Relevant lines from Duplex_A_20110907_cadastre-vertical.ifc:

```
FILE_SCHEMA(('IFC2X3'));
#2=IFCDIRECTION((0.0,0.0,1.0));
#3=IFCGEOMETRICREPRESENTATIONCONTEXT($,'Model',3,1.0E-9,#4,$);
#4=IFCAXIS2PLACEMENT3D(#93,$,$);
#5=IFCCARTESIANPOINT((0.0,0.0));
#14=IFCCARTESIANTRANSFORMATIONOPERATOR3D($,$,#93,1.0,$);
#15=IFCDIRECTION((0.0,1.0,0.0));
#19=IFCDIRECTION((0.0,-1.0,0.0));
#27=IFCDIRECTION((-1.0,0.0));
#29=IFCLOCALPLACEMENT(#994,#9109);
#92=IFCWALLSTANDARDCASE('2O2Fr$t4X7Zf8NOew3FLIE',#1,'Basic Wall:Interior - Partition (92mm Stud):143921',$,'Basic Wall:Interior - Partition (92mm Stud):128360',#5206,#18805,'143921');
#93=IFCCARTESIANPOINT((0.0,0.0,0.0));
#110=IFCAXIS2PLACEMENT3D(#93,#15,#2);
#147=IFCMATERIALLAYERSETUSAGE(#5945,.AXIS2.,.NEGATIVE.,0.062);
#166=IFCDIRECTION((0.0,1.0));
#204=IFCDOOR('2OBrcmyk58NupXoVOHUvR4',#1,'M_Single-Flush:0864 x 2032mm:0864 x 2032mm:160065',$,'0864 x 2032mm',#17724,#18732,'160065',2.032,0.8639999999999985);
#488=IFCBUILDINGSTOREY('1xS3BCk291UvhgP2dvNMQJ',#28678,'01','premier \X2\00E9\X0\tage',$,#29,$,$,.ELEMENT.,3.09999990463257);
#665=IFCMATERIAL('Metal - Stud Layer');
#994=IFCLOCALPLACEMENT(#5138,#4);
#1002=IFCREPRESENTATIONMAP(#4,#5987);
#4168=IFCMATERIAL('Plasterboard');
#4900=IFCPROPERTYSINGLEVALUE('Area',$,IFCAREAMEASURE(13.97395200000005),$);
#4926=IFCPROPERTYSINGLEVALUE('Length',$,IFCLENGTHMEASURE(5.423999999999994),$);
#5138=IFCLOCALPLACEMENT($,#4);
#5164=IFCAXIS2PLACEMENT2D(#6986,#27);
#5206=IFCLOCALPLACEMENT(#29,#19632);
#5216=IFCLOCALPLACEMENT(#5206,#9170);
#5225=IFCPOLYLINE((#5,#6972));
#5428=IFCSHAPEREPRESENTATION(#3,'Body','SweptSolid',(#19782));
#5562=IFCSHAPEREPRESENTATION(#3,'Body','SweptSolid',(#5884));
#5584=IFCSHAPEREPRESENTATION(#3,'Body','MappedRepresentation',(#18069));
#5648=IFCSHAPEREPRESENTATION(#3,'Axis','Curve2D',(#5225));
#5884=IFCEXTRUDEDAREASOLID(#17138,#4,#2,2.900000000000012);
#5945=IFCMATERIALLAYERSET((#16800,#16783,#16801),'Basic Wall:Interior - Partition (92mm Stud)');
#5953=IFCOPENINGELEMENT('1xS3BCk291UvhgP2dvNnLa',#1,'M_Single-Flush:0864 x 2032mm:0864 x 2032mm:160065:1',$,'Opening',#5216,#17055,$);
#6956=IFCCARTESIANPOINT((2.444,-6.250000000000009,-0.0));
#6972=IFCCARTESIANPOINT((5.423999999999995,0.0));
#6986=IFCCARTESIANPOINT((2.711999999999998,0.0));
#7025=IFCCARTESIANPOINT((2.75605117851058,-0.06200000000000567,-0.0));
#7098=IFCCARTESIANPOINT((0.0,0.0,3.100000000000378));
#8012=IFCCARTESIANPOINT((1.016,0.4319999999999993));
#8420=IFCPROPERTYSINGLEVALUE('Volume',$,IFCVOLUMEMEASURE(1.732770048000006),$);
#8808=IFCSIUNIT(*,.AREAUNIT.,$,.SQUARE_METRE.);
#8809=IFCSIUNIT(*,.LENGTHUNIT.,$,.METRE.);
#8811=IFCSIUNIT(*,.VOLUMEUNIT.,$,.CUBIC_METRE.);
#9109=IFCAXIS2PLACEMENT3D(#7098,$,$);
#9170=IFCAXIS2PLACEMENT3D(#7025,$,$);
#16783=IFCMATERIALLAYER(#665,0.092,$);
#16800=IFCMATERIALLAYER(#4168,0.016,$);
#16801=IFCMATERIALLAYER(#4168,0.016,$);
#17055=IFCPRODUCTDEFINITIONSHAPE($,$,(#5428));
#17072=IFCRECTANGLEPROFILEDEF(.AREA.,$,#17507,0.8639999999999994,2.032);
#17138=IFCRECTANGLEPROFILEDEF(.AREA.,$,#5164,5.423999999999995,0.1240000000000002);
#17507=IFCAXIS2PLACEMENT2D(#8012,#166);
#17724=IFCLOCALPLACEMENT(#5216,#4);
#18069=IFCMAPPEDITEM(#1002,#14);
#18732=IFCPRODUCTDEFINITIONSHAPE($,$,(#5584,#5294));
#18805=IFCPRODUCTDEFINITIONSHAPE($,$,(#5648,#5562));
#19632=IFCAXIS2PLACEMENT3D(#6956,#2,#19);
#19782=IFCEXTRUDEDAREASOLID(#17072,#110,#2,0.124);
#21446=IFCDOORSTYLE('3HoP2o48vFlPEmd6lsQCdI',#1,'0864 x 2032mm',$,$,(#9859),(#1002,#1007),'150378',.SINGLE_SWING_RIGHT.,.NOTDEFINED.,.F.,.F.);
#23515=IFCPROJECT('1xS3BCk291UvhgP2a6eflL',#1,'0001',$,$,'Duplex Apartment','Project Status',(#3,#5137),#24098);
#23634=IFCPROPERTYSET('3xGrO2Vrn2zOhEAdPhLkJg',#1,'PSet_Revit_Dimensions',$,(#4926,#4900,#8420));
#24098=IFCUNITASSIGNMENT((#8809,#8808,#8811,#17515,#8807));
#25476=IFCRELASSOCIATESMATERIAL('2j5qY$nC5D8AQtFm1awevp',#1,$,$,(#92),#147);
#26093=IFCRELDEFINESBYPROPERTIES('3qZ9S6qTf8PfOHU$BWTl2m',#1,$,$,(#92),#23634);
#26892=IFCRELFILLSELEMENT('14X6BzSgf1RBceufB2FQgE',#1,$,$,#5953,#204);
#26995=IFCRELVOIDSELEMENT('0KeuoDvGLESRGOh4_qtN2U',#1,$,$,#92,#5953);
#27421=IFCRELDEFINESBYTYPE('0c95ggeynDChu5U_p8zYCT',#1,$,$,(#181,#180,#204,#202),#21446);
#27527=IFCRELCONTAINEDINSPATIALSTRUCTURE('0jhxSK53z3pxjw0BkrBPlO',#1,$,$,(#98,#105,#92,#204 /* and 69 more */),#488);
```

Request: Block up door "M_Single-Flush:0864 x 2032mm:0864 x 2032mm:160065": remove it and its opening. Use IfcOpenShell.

```python
import ifcopenshell
import ifcopenshell.api.feature
import ifcopenshell.api.pset
import ifcopenshell.api.root
import ifcopenshell.geom
import ifcopenshell.util.element
import ifcopenshell.util.shape
import ifcopenshell.util.unit

model = ifcopenshell.open("Duplex_A_20110907_cadastre-vertical.ifc")
area_scale = ifcopenshell.util.unit.calculate_unit_scale(model, "AREAUNIT")
volume_scale = ifcopenshell.util.unit.calculate_unit_scale(model, "VOLUMEUNIT")
settings = ifcopenshell.geom.settings()


def volume(element):
    """Net volume in cubic metres, openings subtracted."""
    shape = ifcopenshell.geom.create_shape(settings, element)
    return ifcopenshell.util.shape.get_volume(shape.geometry)


door = model.by_id(204)
opening = door.FillsVoids[0].RelatingOpeningElement
wall = opening.VoidsElements[0].RelatingBuildingElement
before = volume(wall)

ifcopenshell.api.root.remove_product(model, product=door)
ifcopenshell.api.feature.remove_feature(model, feature=opening)

after = volume(wall)
thickness = 0.124  # wall thickness in metres

# Update the wall's stored quantities.
pset = model.by_id(ifcopenshell.util.element.get_pset(wall, "PSet_Revit_Dimensions", should_inherit=False)["id"])
ifcopenshell.api.pset.edit_pset(model, pset=pset, properties={
    "Area": model.create_entity("IfcAreaMeasure", after / thickness / area_scale),
    "Volume": model.create_entity("IfcVolumeMeasure", after / volume_scale),
})

print(f"wall volume {before:.3f} -> {after:.3f} m3")

model.write("Duplex_A_20110907_cadastre-vertical_v2.ifc")
```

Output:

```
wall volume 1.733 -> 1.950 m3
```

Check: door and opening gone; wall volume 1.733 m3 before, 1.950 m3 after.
